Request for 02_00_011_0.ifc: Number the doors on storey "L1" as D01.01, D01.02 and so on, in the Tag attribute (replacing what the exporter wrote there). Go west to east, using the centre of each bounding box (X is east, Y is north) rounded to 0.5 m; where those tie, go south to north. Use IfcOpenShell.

First a look at what the model holds.

```python
import ifcopenshell
import ifcopenshell.util.element
import ifcopenshell.util.placement

model = ifcopenshell.open("02_00_011_0.ifc")
print(model.schema)
storey = next(s for s in model.by_type("IfcBuildingStorey") if s.Name == "L1")
doors = [e for e in ifcopenshell.util.element.get_decomposition(storey) if e.is_a("IfcDoor")]
for e in sorted(doors, key=lambda e: e.id()):
    origin = ifcopenshell.util.placement.get_local_placement(e.ObjectPlacement)[:3, 3]
    print(e.id(), e.Tag, e.Name, origin.round(2) + 0.0, sep=" | ")
```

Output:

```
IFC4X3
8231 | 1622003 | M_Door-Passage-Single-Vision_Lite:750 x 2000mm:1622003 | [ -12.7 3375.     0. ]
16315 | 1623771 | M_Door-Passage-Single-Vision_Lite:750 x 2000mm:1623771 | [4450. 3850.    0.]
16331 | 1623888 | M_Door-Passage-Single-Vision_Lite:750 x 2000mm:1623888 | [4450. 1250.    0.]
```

```python
import ifcopenshell
import ifcopenshell.geom
import ifcopenshell.util.element
import ifcopenshell.util.shape

model = ifcopenshell.open("02_00_011_0.ifc")
settings = ifcopenshell.geom.settings()
settings.set("use-world-coords", True)


def centre(element):
    shape = ifcopenshell.geom.create_shape(settings, element)
    return ifcopenshell.util.shape.get_bbox_centroid(shape.geometry)


storey = next(s for s in model.by_type("IfcBuildingStorey") if s.Name == "L1")
doors = [e for e in ifcopenshell.util.element.get_decomposition(storey) if e.is_a("IfcDoor")]

# Insertion points can sit at a corner or the storey origin, so sort by the geometry (in metres).
centres = {e: centre(e) for e in doors}
doors.sort(key=lambda e: (round(centres[e][0] / 0.5), centres[e][1]))

for i, e in enumerate(doors, start=1):
    number = f"D01.{i:02d}"
    e.Tag = number
    print(e.id(), number)

model.write("02_00_011_0_edited.ifc")
```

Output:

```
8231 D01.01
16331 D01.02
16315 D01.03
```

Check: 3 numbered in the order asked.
